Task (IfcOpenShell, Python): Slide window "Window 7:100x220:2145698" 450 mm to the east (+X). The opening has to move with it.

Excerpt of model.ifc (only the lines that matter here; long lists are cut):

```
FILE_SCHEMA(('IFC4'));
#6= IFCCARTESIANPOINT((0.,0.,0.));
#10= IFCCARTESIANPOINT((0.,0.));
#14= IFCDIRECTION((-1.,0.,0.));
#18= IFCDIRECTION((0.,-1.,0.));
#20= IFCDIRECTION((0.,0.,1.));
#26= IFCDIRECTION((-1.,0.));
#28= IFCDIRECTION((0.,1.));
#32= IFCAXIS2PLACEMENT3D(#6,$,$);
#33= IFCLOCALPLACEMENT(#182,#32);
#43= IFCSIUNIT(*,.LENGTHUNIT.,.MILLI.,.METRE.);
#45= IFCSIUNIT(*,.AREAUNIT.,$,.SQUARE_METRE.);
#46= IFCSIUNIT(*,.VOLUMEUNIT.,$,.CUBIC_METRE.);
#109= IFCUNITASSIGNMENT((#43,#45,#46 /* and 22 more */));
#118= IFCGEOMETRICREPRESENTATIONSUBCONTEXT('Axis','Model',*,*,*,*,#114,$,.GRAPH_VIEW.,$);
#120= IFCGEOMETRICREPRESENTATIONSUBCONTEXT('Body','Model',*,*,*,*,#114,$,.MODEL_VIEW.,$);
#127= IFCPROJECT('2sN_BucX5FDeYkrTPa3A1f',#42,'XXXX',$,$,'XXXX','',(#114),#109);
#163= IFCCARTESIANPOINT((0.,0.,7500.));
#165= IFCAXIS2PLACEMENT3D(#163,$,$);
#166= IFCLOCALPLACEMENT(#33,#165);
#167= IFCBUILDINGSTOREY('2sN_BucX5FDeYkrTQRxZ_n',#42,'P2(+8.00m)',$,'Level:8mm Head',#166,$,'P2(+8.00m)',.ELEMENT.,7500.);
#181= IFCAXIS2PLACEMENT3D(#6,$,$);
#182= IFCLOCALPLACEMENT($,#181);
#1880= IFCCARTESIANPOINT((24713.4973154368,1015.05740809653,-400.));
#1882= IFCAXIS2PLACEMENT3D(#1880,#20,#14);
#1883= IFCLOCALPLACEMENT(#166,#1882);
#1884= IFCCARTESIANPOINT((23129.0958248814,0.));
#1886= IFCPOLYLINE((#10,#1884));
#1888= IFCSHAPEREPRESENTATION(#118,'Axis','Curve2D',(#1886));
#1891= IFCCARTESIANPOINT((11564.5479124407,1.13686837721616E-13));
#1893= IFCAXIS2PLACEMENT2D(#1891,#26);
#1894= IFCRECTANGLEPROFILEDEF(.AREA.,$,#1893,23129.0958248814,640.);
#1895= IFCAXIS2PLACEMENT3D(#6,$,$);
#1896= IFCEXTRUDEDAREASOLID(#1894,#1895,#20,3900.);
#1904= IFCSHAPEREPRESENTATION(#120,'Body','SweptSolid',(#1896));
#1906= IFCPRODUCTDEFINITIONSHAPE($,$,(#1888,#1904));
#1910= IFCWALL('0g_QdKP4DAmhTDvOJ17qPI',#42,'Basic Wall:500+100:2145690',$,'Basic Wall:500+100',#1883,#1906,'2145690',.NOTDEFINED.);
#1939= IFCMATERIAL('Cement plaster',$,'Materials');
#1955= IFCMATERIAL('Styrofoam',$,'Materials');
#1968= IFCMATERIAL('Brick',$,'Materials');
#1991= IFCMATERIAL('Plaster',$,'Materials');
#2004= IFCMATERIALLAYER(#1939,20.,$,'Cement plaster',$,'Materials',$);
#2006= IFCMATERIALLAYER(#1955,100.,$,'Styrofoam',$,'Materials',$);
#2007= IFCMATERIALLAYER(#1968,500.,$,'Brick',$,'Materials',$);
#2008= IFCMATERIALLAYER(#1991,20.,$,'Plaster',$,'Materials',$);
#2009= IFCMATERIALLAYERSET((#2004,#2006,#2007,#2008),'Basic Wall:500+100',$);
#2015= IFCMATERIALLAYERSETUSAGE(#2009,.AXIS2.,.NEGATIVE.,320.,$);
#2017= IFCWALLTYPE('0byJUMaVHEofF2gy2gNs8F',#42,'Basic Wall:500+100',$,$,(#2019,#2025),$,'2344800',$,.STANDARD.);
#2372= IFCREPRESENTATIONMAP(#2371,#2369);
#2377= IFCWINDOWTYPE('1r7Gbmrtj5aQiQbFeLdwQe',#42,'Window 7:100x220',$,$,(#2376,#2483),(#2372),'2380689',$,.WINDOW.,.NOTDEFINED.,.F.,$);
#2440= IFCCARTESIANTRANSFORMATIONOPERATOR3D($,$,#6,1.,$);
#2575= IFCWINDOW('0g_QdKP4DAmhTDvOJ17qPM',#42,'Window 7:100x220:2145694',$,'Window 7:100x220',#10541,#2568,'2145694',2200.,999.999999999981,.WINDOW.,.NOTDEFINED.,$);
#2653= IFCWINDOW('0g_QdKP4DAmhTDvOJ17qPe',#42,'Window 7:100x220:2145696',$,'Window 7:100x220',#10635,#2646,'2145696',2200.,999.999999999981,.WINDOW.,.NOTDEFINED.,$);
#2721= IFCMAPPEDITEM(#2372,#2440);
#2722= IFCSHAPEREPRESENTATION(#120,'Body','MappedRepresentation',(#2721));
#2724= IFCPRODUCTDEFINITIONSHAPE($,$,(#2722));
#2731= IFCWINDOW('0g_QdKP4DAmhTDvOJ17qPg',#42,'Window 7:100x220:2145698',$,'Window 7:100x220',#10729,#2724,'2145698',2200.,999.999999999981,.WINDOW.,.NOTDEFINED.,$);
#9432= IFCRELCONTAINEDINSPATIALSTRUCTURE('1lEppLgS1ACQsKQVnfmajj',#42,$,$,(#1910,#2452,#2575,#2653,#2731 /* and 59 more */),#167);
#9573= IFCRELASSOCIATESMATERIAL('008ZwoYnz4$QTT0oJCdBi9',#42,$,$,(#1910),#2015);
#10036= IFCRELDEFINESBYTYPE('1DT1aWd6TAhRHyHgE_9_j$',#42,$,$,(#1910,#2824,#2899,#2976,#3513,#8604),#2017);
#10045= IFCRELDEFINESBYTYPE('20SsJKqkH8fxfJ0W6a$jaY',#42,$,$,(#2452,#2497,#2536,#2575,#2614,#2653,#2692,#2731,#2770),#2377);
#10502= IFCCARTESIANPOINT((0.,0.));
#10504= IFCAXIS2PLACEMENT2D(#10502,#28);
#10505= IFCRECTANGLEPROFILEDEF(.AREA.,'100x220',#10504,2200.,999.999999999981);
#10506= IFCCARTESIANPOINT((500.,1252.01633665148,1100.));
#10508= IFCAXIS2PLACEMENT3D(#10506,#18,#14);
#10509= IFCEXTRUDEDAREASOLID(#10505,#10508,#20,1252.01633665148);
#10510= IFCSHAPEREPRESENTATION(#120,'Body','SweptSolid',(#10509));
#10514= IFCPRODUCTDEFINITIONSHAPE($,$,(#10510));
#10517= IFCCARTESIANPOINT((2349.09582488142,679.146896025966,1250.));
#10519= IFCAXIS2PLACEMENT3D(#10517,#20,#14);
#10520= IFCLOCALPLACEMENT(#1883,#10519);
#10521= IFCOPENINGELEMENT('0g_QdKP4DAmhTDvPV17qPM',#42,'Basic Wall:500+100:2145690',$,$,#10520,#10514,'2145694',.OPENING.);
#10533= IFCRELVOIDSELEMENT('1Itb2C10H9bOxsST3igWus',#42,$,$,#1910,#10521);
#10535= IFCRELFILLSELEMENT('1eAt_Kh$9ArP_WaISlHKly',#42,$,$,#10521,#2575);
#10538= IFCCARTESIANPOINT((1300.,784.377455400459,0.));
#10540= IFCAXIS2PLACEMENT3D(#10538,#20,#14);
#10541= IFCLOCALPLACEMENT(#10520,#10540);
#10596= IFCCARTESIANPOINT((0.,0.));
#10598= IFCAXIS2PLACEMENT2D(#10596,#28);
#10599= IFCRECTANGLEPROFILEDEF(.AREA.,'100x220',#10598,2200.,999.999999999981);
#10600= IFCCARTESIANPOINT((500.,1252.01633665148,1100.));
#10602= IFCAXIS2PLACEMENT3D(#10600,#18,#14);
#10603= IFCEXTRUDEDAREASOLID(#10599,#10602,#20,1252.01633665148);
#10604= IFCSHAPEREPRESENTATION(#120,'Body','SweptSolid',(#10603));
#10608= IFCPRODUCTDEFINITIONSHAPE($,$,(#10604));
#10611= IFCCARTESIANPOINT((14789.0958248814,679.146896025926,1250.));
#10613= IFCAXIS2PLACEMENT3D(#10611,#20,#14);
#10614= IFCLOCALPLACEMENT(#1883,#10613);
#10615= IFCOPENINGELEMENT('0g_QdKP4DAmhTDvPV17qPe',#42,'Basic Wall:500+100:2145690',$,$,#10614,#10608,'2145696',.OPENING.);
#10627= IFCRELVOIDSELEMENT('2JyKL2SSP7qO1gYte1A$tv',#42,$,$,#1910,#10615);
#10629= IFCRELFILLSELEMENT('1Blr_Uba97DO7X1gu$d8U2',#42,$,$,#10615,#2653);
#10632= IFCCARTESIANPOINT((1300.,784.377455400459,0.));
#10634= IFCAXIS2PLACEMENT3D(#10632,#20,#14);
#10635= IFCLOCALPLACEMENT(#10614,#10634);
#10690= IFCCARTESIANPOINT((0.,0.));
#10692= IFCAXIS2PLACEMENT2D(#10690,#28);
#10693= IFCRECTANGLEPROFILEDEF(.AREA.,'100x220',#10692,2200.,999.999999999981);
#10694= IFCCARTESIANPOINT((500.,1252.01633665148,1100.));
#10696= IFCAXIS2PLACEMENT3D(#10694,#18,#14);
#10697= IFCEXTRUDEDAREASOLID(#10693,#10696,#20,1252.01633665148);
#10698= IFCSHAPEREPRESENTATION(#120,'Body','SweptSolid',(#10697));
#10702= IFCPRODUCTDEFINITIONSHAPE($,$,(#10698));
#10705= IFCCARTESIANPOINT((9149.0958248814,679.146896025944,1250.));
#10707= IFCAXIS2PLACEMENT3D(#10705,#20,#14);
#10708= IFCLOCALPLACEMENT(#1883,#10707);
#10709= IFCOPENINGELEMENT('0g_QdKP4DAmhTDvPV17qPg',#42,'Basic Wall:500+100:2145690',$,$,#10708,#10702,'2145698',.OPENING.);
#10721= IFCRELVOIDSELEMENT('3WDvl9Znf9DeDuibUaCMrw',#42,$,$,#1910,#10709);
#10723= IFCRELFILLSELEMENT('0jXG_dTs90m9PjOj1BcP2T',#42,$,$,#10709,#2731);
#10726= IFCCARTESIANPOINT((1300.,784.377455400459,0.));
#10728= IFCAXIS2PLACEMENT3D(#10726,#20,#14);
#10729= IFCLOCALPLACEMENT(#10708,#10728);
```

```python
import ifcopenshell
import ifcopenshell.api.geometry
import ifcopenshell.util.placement

model = ifcopenshell.open("model.ifc")

window = model.by_guid("0g_QdKP4DAmhTDvOJ17qPg")
opening = window.FillsVoids[0].RelatingOpeningElement
wall = opening.VoidsElements[0].RelatingBuildingElement

wall_matrix = ifcopenshell.util.placement.get_local_placement(wall.ObjectPlacement)
shift = wall_matrix[:3, 0] * -450.0
before = ifcopenshell.util.placement.get_local_placement(window.ObjectPlacement)[:3, 3].copy()

# The window is placed relative to its opening, so it follows when the opening moves.
matrix = ifcopenshell.util.placement.get_local_placement(opening.ObjectPlacement)
matrix[:3, 3] += shift
ifcopenshell.api.geometry.edit_object_placement(
    model, product=opening, matrix=matrix, is_si=False, should_transform_children=True
)

after = ifcopenshell.util.placement.get_local_placement(window.ObjectPlacement)[:3, 3]
print("window moved by", (after - before).round(3) + 0.0)

model.write("model_v2.ifc")
```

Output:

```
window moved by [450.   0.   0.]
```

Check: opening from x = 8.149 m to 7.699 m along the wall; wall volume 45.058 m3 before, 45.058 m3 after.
